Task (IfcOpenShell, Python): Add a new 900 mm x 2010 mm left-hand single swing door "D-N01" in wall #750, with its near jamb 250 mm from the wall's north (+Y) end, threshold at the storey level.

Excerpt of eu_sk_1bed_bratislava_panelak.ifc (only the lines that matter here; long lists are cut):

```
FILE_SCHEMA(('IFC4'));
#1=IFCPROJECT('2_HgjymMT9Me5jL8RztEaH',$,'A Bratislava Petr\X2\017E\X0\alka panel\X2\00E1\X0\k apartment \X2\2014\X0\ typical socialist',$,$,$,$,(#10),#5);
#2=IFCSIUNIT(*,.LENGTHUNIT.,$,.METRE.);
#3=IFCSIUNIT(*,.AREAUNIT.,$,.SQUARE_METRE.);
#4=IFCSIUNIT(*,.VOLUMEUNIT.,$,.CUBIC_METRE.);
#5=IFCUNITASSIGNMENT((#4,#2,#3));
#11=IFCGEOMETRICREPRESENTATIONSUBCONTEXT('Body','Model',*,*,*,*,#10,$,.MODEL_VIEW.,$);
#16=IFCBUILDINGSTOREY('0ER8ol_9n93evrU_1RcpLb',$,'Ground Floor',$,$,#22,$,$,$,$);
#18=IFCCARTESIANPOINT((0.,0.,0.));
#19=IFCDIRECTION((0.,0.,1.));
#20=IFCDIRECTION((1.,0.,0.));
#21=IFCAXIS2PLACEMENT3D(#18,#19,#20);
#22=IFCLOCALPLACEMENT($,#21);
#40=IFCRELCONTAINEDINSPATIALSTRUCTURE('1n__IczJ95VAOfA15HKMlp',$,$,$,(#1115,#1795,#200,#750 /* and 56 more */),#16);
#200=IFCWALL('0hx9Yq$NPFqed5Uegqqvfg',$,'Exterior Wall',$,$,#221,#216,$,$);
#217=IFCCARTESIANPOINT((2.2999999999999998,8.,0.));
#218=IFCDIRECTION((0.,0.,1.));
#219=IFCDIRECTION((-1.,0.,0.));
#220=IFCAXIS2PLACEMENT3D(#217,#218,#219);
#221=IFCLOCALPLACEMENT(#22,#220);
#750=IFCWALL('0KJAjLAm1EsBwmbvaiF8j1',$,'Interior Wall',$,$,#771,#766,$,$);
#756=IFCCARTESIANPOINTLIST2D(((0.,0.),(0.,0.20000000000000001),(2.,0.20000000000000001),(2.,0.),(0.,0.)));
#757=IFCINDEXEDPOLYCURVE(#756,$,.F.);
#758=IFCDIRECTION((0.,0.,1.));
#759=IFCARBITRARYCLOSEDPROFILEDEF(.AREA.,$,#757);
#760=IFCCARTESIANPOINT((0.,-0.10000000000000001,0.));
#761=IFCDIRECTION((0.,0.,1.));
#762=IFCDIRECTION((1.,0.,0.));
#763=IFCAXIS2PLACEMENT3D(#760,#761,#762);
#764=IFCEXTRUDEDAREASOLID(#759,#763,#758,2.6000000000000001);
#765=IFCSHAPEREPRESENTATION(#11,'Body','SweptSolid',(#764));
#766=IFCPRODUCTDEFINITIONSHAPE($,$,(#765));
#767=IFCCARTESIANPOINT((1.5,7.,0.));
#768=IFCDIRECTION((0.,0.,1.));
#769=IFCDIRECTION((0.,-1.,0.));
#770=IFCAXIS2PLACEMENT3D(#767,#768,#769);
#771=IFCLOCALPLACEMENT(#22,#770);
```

```python
import numpy as np
import ifcopenshell
import ifcopenshell.api.feature
import ifcopenshell.api.geometry
import ifcopenshell.api.root
import ifcopenshell.api.spatial
import ifcopenshell.geom
import ifcopenshell.util.element
import ifcopenshell.util.placement
import ifcopenshell.util.representation
import ifcopenshell.util.shape
import ifcopenshell.util.unit

model = ifcopenshell.open("eu_sk_1bed_bratislava_panelak.ifc")
unit_scale = ifcopenshell.util.unit.calculate_unit_scale(model)
settings = ifcopenshell.geom.settings()


def volume(element):
    """Net volume in cubic metres, openings subtracted."""
    shape = ifcopenshell.geom.create_shape(settings, element)
    return ifcopenshell.util.shape.get_volume(shape.geometry)


wall = model.by_guid("0KJAjLAm1EsBwmbvaiF8j1")
storey = ifcopenshell.util.element.get_container(wall, ifc_class="IfcBuildingStorey")
context = ifcopenshell.util.representation.get_context(model, "Model", "Body", "MODEL_VIEW")
before = volume(wall)

width, height, from_end, sill = 0.9, 2.01, 0.25, 0.0  # metres

# The wall runs along its own X axis, and the end named is its -X end.
wall_shape = ifcopenshell.geom.create_shape(settings, wall)
x, y, z = ifcopenshell.util.shape.get_vertices(wall_shape.geometry).T
start = x.min() + from_end
face, thickness = float(y.min()), float(y.max() - y.min())
wall_matrix = ifcopenshell.util.placement.get_local_placement(wall.ObjectPlacement)
level = ifcopenshell.util.placement.get_local_placement(storey.ObjectPlacement)[2, 3]


def in_wall(x, y):
    """Placement at x, y metres in the wall's axes, at sill height."""
    matrix = wall_matrix.copy()
    matrix[:, 3] = wall_matrix @ np.array([x / unit_scale, y / unit_scale, 0.0, 1.0])
    matrix[2, 3] = level + sill / unit_scale
    return matrix


# Opening: a box that overshoots both wall faces by 50 mm.
opening = ifcopenshell.api.root.create_entity(model, ifc_class="IfcOpeningElement", predefined_type="OPENING")
box = ifcopenshell.api.geometry.add_wall_representation(
    model, context=context, length=width, height=height, thickness=thickness + 0.1
)
ifcopenshell.api.geometry.assign_representation(model, product=opening, representation=box)
ifcopenshell.api.geometry.edit_object_placement(model, product=opening, matrix=in_wall(start, face - 0.05), is_si=False)
ifcopenshell.api.feature.add_feature(model, feature=opening, element=wall)

door = ifcopenshell.api.root.create_entity(model, ifc_class="IfcDoor", name="D-N01", predefined_type="DOOR")
door.OverallWidth, door.OverallHeight = width / unit_scale, height / unit_scale
door.OperationType = "SINGLE_SWING_LEFT"
body = ifcopenshell.api.geometry.add_door_representation(
    model,
    context=context,
    overall_width=door.OverallWidth,
    overall_height=door.OverallHeight,
    operation_type="SINGLE_SWING_LEFT",
    lining_properties={"LiningDepth": thickness / unit_scale, "ThresholdDepth": thickness / unit_scale},
)
ifcopenshell.api.geometry.assign_representation(model, product=door, representation=body)
ifcopenshell.api.spatial.assign_container(model, products=[door], relating_structure=storey)
ifcopenshell.api.feature.add_filling(model, opening=opening, element=door)

# The lining spans the wall, so the door starts at the wall face.
ifcopenshell.api.geometry.edit_object_placement(model, product=door, matrix=in_wall(start, face), is_si=False)

after = volume(wall)

print(f"wall volume {before:.3f} -> {after:.3f} m3")

model.write("eu_sk_1bed_bratislava_panelak_edited.ifc")
```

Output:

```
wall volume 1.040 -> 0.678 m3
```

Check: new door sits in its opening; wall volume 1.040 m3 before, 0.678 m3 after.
